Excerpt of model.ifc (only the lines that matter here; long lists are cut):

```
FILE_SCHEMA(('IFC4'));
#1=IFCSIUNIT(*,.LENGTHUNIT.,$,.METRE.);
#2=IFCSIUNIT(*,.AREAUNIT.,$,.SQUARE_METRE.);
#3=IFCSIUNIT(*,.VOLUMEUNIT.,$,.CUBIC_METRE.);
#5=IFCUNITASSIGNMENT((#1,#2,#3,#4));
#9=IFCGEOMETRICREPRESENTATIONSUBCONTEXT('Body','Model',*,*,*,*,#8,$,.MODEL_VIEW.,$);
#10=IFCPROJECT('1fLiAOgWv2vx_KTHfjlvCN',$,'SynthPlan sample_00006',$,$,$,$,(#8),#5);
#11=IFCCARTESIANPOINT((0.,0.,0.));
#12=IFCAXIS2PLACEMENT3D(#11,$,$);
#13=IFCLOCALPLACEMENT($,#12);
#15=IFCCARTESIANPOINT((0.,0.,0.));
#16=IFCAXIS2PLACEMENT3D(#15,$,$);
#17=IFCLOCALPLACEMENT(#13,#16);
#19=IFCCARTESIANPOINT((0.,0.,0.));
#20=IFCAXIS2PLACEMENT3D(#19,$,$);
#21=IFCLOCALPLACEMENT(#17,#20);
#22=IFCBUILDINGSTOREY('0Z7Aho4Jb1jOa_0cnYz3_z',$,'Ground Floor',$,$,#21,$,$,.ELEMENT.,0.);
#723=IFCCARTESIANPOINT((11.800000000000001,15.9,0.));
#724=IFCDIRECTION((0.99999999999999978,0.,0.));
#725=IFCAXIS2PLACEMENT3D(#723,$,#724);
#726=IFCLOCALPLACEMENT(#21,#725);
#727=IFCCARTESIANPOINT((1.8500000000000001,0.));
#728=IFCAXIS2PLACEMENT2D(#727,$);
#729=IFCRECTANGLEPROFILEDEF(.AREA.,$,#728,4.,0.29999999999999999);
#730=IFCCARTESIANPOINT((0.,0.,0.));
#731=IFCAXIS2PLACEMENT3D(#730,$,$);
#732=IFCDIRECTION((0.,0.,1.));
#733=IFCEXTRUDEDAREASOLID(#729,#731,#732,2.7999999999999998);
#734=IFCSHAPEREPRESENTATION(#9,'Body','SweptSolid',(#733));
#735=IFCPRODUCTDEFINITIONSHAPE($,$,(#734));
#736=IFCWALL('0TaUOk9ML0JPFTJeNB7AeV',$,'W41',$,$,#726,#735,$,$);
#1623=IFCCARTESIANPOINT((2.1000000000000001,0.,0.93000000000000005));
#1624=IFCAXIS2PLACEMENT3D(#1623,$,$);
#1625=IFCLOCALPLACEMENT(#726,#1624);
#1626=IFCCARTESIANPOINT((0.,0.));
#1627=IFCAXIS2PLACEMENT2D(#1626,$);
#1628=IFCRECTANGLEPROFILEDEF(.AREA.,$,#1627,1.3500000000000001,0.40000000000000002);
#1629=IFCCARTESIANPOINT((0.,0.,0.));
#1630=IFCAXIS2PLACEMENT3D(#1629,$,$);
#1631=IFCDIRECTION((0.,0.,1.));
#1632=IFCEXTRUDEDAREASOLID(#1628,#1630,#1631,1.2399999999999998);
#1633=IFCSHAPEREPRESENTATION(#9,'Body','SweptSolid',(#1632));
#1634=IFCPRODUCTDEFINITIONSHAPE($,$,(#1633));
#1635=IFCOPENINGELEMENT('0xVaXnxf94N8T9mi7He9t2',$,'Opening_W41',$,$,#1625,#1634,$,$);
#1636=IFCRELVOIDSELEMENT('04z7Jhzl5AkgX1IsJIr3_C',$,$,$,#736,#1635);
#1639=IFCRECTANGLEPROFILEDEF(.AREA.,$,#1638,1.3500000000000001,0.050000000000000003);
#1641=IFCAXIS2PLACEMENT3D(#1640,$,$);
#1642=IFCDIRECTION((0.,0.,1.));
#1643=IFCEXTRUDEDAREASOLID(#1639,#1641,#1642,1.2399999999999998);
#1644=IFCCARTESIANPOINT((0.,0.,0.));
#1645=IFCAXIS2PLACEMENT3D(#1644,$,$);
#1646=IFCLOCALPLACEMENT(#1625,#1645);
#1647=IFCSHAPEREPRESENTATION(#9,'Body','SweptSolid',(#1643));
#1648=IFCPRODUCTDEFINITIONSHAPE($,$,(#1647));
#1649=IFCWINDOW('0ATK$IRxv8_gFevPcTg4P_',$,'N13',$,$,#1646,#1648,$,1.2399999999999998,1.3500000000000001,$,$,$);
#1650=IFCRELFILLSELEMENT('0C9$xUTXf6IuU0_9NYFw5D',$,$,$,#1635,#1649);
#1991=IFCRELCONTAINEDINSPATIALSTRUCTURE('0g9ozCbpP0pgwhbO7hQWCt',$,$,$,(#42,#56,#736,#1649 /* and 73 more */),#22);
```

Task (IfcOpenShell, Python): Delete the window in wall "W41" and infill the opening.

```python
import ifcopenshell
import ifcopenshell.api.feature
import ifcopenshell.api.root
import ifcopenshell.geom
import ifcopenshell.util.shape

model = ifcopenshell.open("model.ifc")
settings = ifcopenshell.geom.settings()


def volume(element):
    """Net volume in cubic metres, openings subtracted."""
    shape = ifcopenshell.geom.create_shape(settings, element)
    return ifcopenshell.util.shape.get_volume(shape.geometry)


window = model.by_guid("0ATK$IRxv8_gFevPcTg4P_")
opening = window.FillsVoids[0].RelatingOpeningElement
wall = opening.VoidsElements[0].RelatingBuildingElement
before = volume(wall)

ifcopenshell.api.root.remove_product(model, product=window)
ifcopenshell.api.feature.remove_feature(model, feature=opening)

after = volume(wall)

print(f"wall volume {before:.3f} -> {after:.3f} m3")

model.write("model-out.ifc")
```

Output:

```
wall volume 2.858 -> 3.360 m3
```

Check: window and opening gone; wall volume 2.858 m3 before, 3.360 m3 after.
